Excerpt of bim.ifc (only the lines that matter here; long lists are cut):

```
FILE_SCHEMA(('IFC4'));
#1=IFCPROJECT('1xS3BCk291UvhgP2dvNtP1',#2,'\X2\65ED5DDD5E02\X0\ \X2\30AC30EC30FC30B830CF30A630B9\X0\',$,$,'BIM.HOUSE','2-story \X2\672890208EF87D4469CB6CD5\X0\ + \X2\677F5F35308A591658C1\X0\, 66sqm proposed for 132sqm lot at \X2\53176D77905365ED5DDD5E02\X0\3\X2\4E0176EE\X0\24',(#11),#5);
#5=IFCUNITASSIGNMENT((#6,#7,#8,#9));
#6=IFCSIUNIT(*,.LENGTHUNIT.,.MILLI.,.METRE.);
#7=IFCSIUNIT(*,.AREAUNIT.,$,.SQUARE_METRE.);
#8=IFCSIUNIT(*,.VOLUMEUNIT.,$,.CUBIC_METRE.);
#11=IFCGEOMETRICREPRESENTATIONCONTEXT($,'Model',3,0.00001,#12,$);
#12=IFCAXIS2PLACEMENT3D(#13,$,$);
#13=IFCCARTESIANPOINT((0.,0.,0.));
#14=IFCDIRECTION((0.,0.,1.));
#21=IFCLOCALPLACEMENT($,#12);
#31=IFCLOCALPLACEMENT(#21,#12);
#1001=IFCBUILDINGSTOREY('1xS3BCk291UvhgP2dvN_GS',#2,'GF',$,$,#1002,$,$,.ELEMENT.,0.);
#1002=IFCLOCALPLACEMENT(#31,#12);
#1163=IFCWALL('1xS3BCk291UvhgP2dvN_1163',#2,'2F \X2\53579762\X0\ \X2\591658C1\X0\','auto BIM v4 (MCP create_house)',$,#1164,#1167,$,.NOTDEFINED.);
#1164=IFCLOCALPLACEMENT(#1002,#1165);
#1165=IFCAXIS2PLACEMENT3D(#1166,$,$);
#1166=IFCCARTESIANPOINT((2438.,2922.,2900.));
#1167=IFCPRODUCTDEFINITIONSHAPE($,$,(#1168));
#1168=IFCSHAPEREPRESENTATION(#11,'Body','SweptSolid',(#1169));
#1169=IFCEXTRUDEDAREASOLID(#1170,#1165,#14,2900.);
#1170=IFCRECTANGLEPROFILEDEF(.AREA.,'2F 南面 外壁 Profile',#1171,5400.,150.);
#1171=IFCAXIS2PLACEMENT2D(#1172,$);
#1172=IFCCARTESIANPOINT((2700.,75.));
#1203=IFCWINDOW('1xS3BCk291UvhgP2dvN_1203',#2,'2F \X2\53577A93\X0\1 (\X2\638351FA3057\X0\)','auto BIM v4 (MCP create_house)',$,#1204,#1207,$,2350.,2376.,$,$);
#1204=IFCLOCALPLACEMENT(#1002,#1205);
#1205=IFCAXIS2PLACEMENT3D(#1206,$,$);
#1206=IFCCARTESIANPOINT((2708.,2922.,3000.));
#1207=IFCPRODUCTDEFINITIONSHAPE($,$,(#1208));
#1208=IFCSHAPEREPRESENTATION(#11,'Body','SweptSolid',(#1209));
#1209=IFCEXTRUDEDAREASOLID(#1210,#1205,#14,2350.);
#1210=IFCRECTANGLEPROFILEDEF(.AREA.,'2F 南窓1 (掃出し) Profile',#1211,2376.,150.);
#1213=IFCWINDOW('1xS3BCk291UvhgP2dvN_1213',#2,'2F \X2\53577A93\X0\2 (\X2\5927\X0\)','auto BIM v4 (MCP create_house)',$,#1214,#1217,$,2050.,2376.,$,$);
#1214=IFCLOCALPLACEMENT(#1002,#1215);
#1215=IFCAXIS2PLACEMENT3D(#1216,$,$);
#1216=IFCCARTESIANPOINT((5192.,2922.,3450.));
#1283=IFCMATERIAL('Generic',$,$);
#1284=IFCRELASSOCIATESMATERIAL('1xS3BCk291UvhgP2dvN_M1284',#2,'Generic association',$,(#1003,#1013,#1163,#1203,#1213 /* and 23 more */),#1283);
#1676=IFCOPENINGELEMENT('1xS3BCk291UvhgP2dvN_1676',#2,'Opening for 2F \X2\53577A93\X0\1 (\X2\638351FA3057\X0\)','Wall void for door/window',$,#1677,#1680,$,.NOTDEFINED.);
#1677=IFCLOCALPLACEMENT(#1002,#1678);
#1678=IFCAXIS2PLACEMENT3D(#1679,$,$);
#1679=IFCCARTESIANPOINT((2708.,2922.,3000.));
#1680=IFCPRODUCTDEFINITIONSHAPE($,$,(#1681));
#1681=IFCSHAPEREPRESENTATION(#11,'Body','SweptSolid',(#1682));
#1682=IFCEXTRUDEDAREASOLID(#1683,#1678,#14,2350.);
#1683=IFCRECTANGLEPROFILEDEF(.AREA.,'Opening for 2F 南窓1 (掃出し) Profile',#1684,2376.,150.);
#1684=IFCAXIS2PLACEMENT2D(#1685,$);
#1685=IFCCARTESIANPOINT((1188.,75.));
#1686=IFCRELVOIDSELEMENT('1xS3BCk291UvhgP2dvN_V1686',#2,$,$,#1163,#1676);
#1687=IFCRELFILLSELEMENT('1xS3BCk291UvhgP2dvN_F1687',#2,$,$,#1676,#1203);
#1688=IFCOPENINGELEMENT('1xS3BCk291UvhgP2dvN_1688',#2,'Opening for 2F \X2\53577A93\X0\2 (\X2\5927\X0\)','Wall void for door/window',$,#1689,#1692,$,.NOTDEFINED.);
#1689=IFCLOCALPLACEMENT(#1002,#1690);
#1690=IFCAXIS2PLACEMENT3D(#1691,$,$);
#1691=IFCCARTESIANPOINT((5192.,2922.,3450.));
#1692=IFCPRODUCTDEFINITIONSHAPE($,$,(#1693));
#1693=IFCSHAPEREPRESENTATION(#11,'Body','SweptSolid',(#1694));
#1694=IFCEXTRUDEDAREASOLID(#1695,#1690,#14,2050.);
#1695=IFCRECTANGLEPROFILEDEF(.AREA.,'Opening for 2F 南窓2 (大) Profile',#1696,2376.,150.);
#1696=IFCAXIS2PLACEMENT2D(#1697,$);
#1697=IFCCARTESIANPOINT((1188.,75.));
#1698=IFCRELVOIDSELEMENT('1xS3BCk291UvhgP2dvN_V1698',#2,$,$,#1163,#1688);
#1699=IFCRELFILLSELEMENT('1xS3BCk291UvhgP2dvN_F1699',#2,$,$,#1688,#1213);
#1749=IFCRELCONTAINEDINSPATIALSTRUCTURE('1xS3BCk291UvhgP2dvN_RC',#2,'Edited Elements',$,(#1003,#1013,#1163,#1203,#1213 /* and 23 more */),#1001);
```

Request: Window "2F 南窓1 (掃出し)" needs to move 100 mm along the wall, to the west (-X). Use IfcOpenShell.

```python
import ifcopenshell
import ifcopenshell.api.geometry
import ifcopenshell.util.placement
import ifcopenshell.util.unit

model = ifcopenshell.open("bim.ifc")
unit_scale = ifcopenshell.util.unit.calculate_unit_scale(model)

window = model.by_id(1203)
opening = window.FillsVoids[0].RelatingOpeningElement
wall = opening.VoidsElements[0].RelatingBuildingElement

wall_matrix = ifcopenshell.util.placement.get_local_placement(wall.ObjectPlacement)
shift = wall_matrix[:3, 0] * -0.1 / unit_scale
before = ifcopenshell.util.placement.get_local_placement(window.ObjectPlacement)[:3, 3].copy()

# The window is not placed relative to its opening, so move both.
for product in (opening, window):
    matrix = ifcopenshell.util.placement.get_local_placement(product.ObjectPlacement)
    matrix[:3, 3] += shift
    ifcopenshell.api.geometry.edit_object_placement(model, product=product, matrix=matrix, is_si=False)

after = ifcopenshell.util.placement.get_local_placement(window.ObjectPlacement)[:3, 3]
print("window moved by", (after - before).round(3) + 0.0)

model.write("bim-out.ifc")
```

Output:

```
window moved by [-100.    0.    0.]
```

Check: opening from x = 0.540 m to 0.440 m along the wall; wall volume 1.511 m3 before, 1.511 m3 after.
